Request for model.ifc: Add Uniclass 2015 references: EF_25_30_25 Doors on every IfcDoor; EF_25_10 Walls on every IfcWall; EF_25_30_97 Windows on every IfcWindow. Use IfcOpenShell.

First a look at what the model holds.

```python
import ifcopenshell

model = ifcopenshell.open("model.ifc")
print(model.schema)
print("classifications:", [c.Name for c in model.by_type("IfcClassification")])
for ifc_class in ("IfcDoor", "IfcRoof", "IfcStair", "IfcWall", "IfcWindow"):
    print(ifc_class, len(model.by_type(ifc_class)))
```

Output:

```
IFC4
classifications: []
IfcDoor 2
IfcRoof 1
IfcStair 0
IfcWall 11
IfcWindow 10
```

```python
import ifcopenshell
import ifcopenshell.api.classification

model = ifcopenshell.open("model.ifc")

system = ifcopenshell.api.classification.add_classification(model, classification="Uniclass 2015")

codes = {
    "IfcDoor": ("EF_25_30_25", "Doors"),
    "IfcWall": ("EF_25_10", "Walls"),
    "IfcWindow": ("EF_25_30_97", "Windows"),
}
for ifc_class, (code, name) in codes.items():
    products = model.by_type(ifc_class)
    ifcopenshell.api.classification.add_reference(
        model, products=products, classification=system, identification=code, name=name
    )
    print(code, len(products))

model.write("model_rev.ifc")
```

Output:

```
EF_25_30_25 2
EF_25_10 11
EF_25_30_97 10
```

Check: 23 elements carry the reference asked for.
